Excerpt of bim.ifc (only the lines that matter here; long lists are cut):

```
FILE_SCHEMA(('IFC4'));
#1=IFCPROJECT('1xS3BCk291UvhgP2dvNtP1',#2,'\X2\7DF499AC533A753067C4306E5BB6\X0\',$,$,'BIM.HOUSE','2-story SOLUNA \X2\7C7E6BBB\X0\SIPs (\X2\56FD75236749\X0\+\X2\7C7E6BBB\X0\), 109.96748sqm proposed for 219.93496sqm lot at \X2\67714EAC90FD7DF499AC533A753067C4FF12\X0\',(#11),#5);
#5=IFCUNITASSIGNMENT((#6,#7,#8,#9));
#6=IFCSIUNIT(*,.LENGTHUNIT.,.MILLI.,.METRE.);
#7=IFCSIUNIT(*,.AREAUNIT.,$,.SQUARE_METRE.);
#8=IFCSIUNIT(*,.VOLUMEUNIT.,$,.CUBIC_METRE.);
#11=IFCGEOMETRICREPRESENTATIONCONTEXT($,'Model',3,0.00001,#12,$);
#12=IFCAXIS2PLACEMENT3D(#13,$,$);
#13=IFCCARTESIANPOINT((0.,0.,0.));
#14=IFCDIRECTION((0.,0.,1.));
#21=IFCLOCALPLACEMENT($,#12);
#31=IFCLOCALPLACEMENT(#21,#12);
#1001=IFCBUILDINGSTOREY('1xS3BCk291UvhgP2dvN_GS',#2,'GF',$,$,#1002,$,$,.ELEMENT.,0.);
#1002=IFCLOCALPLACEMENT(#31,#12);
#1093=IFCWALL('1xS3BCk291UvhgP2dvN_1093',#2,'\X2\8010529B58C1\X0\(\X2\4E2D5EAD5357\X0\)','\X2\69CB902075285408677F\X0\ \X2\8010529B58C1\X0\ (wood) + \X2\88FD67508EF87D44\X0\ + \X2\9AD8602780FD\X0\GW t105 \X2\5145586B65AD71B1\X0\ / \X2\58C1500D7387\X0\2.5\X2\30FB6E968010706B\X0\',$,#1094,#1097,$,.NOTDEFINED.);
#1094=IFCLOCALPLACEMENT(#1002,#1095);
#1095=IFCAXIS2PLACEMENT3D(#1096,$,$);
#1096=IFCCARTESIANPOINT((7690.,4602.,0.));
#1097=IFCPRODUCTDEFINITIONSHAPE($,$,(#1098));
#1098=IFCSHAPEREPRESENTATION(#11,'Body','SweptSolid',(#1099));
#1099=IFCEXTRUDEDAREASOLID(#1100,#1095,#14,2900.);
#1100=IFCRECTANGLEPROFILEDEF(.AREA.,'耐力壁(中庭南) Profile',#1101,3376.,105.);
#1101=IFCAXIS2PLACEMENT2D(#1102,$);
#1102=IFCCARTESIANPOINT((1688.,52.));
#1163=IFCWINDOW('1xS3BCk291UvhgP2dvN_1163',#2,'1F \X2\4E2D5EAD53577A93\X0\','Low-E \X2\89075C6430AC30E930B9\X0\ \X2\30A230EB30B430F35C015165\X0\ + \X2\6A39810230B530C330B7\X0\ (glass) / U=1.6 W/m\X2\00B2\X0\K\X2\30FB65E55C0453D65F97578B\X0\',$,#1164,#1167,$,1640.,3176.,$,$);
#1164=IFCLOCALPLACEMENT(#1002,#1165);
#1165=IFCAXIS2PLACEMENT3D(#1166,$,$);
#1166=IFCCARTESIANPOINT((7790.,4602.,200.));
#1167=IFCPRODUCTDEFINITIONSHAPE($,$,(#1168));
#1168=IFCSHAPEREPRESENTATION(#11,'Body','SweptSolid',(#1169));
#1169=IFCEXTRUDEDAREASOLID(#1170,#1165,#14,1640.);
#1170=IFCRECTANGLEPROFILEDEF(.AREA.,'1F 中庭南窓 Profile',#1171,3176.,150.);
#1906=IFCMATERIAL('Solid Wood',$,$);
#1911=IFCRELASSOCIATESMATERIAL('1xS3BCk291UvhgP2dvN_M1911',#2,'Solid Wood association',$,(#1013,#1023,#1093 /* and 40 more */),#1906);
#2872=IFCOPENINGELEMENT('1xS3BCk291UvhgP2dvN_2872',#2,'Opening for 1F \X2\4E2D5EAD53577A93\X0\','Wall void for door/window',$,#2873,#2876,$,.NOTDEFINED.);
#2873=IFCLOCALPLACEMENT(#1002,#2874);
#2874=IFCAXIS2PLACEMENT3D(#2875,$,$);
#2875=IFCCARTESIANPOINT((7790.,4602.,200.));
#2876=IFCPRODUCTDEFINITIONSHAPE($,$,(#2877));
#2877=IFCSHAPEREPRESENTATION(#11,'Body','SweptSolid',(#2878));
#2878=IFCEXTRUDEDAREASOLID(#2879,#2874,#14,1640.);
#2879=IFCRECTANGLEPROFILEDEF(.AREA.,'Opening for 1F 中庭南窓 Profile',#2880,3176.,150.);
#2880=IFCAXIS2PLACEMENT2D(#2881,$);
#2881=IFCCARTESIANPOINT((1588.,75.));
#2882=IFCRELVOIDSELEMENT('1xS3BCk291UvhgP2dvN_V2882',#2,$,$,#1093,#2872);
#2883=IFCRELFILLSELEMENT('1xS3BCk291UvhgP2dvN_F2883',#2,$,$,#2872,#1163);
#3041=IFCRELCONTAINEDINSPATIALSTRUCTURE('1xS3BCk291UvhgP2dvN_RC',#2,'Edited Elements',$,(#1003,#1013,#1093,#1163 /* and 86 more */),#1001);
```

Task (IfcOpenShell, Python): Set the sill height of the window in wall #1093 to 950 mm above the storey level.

```python
import numpy as np
import ifcopenshell
import ifcopenshell.api.geometry
import ifcopenshell.geom
import ifcopenshell.util.element
import ifcopenshell.util.placement
import ifcopenshell.util.shape
import ifcopenshell.util.unit

model = ifcopenshell.open("bim.ifc")
unit_scale = ifcopenshell.util.unit.calculate_unit_scale(model)

window = model.by_guid("1xS3BCk291UvhgP2dvN_1163")
opening = window.FillsVoids[0].RelatingOpeningElement
storey = ifcopenshell.util.element.get_container(window, ifc_class="IfcBuildingStorey")
level = ifcopenshell.util.placement.get_local_placement(storey.ObjectPlacement)[2, 3]

# The opening's origin need not be at the sill, so measure its lowest point.
shape = ifcopenshell.geom.create_shape(ifcopenshell.geom.settings(), opening)
bottom = ifcopenshell.util.shape.get_shape_bottom_elevation(shape, shape.geometry) / unit_scale
dz = level + 950.0 - bottom

shift = np.array([0.0, 0.0, dz])
# The window is not placed relative to its opening, so move both.
for product in (opening, window):
    matrix = ifcopenshell.util.placement.get_local_placement(product.ObjectPlacement)
    matrix[:3, 3] += shift
    ifcopenshell.api.geometry.edit_object_placement(model, product=product, matrix=matrix, is_si=False)

print(f"moved by {dz * unit_scale:+.3f} m")

model.write("bim_rev.ifc")
```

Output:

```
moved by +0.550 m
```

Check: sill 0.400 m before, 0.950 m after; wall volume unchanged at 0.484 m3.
